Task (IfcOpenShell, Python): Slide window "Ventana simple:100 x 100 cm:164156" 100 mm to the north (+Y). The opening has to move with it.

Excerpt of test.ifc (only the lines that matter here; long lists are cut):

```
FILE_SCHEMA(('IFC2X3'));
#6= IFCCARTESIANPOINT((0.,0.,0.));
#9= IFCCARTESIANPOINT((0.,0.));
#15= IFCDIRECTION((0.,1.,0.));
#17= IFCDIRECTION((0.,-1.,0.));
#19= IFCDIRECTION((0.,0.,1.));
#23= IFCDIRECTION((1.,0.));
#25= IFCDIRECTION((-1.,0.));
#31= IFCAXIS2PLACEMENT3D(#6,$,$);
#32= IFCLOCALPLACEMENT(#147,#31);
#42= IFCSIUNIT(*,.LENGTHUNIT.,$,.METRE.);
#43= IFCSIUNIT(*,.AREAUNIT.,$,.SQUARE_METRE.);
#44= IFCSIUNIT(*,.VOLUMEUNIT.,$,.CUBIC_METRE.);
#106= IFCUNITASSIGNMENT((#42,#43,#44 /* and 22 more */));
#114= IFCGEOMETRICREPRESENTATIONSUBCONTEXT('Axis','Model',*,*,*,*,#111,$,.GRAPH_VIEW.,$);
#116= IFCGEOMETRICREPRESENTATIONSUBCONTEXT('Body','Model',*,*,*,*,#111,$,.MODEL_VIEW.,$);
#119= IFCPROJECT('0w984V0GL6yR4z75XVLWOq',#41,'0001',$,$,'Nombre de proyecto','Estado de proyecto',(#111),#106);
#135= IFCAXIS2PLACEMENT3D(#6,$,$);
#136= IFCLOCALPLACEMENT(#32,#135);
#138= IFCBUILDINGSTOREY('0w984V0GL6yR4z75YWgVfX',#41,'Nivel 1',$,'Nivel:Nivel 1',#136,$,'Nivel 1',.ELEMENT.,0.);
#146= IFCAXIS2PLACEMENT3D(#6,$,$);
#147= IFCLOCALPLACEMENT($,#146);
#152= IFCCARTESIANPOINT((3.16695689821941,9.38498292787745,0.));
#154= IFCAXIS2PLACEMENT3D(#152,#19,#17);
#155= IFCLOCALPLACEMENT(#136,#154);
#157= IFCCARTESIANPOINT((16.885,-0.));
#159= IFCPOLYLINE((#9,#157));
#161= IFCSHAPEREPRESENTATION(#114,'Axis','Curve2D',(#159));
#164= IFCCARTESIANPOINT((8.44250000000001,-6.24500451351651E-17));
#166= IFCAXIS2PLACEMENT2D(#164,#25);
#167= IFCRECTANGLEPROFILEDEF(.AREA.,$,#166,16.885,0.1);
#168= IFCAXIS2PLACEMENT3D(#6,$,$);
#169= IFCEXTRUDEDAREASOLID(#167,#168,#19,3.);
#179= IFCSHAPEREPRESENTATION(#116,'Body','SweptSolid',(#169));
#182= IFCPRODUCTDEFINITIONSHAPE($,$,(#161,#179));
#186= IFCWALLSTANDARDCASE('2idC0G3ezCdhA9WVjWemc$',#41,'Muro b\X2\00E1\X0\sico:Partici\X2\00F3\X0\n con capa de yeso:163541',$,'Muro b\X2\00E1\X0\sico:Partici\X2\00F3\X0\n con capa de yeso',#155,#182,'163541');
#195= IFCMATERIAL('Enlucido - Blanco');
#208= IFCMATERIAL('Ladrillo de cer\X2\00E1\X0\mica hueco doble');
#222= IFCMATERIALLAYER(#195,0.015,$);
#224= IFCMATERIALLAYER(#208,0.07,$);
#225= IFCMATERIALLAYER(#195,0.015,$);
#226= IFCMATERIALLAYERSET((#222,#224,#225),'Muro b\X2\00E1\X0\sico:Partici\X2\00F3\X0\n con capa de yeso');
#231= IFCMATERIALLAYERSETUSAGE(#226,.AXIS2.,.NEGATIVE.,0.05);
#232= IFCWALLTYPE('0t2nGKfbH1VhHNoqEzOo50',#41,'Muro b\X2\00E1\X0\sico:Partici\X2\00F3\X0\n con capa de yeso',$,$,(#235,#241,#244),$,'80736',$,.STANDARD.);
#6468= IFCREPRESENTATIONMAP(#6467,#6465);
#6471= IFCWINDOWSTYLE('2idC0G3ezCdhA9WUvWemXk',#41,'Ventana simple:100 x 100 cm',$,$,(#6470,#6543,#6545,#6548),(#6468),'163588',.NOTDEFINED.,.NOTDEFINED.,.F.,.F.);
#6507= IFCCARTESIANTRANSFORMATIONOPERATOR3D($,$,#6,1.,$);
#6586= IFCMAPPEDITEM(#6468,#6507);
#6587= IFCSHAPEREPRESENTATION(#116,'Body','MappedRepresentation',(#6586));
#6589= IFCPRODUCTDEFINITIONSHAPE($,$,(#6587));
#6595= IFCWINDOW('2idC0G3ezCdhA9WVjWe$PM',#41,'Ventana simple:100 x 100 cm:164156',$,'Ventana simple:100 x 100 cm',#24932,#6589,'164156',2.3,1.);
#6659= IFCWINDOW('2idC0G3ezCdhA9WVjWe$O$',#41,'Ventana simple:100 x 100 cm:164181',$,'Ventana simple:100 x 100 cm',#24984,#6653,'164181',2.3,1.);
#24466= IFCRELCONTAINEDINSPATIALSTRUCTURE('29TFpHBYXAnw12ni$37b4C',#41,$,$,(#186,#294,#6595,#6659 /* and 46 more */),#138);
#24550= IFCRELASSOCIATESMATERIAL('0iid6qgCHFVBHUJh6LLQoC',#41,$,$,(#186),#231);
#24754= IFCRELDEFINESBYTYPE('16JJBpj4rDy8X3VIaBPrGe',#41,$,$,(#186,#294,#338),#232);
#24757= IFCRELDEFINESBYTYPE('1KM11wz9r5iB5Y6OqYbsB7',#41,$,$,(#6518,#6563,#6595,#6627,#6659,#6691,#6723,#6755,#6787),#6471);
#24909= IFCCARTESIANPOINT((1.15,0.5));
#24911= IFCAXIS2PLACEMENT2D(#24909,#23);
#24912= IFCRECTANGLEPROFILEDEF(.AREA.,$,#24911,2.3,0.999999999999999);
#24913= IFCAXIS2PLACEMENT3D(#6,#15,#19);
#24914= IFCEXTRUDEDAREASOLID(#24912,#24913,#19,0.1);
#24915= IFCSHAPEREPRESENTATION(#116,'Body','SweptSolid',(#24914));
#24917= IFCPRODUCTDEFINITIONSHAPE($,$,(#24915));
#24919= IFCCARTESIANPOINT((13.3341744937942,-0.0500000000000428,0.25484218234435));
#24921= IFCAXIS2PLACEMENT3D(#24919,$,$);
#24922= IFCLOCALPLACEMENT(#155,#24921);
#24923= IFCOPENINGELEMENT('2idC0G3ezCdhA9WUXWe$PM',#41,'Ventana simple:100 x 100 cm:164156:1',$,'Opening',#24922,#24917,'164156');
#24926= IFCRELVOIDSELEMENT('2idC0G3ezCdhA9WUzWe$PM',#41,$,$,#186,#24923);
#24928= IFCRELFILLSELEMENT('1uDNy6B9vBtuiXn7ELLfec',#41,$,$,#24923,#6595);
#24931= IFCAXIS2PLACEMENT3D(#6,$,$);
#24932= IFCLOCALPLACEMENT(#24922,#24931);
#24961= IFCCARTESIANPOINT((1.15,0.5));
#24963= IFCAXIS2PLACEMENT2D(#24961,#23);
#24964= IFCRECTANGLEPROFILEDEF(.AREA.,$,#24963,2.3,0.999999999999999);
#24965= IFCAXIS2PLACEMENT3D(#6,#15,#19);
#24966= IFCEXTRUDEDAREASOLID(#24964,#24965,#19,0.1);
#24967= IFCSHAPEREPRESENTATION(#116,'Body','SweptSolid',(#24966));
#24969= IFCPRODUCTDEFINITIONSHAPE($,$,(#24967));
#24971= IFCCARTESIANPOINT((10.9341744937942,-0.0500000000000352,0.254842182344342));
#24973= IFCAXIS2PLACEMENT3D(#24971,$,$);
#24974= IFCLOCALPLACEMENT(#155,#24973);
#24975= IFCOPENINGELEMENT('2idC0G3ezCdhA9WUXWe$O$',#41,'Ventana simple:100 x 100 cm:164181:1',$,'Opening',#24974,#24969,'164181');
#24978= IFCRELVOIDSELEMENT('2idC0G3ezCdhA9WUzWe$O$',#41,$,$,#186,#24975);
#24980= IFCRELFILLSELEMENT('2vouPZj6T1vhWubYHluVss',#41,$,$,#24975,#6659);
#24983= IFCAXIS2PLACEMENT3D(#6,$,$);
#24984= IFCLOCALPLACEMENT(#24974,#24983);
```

```python
import ifcopenshell
import ifcopenshell.api.geometry
import ifcopenshell.util.placement
import ifcopenshell.util.unit

model = ifcopenshell.open("test.ifc")
unit_scale = ifcopenshell.util.unit.calculate_unit_scale(model)

window = model.by_guid("2idC0G3ezCdhA9WVjWe$PM")
opening = window.FillsVoids[0].RelatingOpeningElement
wall = opening.VoidsElements[0].RelatingBuildingElement

wall_matrix = ifcopenshell.util.placement.get_local_placement(wall.ObjectPlacement)
shift = wall_matrix[:3, 0] * -0.1 / unit_scale
before = ifcopenshell.util.placement.get_local_placement(window.ObjectPlacement)[:3, 3].copy()

# The window is placed relative to its opening, so it follows when the opening moves.
matrix = ifcopenshell.util.placement.get_local_placement(opening.ObjectPlacement)
matrix[:3, 3] += shift
ifcopenshell.api.geometry.edit_object_placement(
    model, product=opening, matrix=matrix, is_si=False, should_transform_children=True
)

after = ifcopenshell.util.placement.get_local_placement(window.ObjectPlacement)[:3, 3]
print("window moved by", (after - before).round(3) + 0.0)

model.write("test_updated.ifc")
```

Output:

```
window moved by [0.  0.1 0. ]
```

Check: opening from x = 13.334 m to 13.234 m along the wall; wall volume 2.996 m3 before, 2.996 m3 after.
